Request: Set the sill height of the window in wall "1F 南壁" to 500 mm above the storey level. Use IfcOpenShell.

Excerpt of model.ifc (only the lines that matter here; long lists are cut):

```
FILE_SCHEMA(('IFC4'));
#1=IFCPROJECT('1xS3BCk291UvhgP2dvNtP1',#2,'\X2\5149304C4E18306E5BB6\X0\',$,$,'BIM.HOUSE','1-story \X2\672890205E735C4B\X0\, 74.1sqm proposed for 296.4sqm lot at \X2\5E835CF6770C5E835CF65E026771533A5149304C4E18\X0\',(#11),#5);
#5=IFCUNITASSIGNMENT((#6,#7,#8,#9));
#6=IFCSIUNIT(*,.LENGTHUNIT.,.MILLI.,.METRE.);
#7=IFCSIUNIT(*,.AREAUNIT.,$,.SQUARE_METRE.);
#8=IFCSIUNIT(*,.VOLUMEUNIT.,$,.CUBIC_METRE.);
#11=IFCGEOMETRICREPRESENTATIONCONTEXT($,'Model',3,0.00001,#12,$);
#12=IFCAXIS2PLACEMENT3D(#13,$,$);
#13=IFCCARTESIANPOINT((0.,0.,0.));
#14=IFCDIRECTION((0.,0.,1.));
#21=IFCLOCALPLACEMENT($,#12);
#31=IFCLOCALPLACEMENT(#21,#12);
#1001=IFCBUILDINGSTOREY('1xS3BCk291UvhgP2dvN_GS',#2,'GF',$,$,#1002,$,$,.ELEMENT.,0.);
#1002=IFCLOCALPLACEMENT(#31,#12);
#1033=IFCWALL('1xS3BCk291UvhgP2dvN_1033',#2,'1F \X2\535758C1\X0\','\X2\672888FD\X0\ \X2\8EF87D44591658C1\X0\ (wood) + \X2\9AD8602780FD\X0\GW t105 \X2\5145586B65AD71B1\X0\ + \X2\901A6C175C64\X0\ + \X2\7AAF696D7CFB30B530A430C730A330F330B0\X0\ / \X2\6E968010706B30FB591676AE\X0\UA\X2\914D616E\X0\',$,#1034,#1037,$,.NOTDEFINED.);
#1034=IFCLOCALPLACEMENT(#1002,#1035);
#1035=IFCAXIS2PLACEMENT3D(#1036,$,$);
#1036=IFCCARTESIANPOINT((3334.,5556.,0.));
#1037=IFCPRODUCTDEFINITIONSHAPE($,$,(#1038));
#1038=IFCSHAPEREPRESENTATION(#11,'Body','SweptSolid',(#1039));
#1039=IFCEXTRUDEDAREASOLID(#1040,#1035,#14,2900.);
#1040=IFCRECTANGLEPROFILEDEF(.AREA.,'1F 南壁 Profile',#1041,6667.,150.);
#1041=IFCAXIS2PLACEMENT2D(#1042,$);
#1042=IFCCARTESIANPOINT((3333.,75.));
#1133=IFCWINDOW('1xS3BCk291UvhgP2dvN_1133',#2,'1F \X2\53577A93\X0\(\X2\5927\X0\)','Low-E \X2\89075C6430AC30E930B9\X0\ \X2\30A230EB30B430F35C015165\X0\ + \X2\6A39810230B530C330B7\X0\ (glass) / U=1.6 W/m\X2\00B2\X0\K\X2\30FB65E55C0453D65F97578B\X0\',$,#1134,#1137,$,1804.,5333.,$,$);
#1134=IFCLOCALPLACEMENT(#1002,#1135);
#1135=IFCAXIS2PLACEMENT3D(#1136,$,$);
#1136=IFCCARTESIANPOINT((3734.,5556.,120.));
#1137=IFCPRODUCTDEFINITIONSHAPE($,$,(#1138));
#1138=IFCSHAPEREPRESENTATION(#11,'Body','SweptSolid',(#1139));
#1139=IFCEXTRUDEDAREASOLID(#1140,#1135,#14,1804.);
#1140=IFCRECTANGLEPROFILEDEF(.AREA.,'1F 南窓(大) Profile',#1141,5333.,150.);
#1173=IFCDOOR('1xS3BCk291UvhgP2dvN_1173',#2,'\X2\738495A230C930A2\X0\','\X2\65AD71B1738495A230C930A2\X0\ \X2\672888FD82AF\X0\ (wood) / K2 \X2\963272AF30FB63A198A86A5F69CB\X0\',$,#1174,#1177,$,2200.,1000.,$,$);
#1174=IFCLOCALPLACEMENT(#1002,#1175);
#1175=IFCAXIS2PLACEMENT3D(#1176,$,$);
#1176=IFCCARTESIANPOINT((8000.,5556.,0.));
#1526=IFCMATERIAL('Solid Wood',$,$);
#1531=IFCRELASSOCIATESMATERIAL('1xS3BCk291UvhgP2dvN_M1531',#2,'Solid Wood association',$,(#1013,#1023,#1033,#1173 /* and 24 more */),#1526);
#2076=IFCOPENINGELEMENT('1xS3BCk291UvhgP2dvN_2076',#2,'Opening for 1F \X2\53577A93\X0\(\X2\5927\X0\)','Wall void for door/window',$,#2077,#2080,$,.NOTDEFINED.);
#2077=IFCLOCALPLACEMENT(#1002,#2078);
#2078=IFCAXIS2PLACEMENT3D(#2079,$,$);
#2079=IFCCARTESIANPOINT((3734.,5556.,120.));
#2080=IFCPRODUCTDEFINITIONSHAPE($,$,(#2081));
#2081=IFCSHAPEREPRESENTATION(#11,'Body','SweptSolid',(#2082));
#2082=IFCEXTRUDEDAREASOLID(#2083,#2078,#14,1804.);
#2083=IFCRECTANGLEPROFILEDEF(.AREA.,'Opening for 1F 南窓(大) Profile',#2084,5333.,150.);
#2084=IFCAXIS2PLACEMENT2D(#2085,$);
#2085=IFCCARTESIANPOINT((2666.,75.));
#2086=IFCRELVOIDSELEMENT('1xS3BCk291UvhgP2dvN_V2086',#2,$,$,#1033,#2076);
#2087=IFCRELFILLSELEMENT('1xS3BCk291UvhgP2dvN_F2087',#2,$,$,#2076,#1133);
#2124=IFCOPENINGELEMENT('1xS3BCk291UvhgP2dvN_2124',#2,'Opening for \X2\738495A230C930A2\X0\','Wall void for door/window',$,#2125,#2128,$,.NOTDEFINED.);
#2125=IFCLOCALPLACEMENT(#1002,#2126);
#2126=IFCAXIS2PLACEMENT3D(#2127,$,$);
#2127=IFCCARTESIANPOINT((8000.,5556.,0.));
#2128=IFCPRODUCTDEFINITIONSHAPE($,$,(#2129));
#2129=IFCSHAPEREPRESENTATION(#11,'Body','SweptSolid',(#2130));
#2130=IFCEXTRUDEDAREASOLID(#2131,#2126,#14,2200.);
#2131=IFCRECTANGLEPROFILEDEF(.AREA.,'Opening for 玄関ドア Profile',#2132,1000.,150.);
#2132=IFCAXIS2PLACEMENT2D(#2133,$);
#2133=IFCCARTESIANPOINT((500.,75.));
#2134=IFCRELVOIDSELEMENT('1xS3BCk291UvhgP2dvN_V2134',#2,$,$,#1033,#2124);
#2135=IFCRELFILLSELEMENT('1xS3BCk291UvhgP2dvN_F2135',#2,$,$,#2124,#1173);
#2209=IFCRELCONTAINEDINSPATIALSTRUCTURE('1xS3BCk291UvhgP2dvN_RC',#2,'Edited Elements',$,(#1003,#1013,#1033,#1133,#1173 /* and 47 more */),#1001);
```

```python
import numpy as np
import ifcopenshell
import ifcopenshell.api.geometry
import ifcopenshell.geom
import ifcopenshell.util.element
import ifcopenshell.util.placement
import ifcopenshell.util.shape
import ifcopenshell.util.unit

model = ifcopenshell.open("model.ifc")
unit_scale = ifcopenshell.util.unit.calculate_unit_scale(model)

window = model.by_guid("1xS3BCk291UvhgP2dvN_1133")
opening = window.FillsVoids[0].RelatingOpeningElement
storey = ifcopenshell.util.element.get_container(window, ifc_class="IfcBuildingStorey")
level = ifcopenshell.util.placement.get_local_placement(storey.ObjectPlacement)[2, 3]

# The opening's origin need not be at the sill, so measure its lowest point.
shape = ifcopenshell.geom.create_shape(ifcopenshell.geom.settings(), opening)
bottom = ifcopenshell.util.shape.get_shape_bottom_elevation(shape, shape.geometry) / unit_scale
dz = level + 0.5 / unit_scale - bottom

shift = np.array([0.0, 0.0, dz])
# The window is not placed relative to its opening, so move both.
for product in (opening, window):
    matrix = ifcopenshell.util.placement.get_local_placement(product.ObjectPlacement)
    matrix[:3, 3] += shift
    ifcopenshell.api.geometry.edit_object_placement(model, product=product, matrix=matrix, is_si=False)

print(f"moved by {dz * unit_scale:+.3f} m")

model.write("model-out.ifc")
```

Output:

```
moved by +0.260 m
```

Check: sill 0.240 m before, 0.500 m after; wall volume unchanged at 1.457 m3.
